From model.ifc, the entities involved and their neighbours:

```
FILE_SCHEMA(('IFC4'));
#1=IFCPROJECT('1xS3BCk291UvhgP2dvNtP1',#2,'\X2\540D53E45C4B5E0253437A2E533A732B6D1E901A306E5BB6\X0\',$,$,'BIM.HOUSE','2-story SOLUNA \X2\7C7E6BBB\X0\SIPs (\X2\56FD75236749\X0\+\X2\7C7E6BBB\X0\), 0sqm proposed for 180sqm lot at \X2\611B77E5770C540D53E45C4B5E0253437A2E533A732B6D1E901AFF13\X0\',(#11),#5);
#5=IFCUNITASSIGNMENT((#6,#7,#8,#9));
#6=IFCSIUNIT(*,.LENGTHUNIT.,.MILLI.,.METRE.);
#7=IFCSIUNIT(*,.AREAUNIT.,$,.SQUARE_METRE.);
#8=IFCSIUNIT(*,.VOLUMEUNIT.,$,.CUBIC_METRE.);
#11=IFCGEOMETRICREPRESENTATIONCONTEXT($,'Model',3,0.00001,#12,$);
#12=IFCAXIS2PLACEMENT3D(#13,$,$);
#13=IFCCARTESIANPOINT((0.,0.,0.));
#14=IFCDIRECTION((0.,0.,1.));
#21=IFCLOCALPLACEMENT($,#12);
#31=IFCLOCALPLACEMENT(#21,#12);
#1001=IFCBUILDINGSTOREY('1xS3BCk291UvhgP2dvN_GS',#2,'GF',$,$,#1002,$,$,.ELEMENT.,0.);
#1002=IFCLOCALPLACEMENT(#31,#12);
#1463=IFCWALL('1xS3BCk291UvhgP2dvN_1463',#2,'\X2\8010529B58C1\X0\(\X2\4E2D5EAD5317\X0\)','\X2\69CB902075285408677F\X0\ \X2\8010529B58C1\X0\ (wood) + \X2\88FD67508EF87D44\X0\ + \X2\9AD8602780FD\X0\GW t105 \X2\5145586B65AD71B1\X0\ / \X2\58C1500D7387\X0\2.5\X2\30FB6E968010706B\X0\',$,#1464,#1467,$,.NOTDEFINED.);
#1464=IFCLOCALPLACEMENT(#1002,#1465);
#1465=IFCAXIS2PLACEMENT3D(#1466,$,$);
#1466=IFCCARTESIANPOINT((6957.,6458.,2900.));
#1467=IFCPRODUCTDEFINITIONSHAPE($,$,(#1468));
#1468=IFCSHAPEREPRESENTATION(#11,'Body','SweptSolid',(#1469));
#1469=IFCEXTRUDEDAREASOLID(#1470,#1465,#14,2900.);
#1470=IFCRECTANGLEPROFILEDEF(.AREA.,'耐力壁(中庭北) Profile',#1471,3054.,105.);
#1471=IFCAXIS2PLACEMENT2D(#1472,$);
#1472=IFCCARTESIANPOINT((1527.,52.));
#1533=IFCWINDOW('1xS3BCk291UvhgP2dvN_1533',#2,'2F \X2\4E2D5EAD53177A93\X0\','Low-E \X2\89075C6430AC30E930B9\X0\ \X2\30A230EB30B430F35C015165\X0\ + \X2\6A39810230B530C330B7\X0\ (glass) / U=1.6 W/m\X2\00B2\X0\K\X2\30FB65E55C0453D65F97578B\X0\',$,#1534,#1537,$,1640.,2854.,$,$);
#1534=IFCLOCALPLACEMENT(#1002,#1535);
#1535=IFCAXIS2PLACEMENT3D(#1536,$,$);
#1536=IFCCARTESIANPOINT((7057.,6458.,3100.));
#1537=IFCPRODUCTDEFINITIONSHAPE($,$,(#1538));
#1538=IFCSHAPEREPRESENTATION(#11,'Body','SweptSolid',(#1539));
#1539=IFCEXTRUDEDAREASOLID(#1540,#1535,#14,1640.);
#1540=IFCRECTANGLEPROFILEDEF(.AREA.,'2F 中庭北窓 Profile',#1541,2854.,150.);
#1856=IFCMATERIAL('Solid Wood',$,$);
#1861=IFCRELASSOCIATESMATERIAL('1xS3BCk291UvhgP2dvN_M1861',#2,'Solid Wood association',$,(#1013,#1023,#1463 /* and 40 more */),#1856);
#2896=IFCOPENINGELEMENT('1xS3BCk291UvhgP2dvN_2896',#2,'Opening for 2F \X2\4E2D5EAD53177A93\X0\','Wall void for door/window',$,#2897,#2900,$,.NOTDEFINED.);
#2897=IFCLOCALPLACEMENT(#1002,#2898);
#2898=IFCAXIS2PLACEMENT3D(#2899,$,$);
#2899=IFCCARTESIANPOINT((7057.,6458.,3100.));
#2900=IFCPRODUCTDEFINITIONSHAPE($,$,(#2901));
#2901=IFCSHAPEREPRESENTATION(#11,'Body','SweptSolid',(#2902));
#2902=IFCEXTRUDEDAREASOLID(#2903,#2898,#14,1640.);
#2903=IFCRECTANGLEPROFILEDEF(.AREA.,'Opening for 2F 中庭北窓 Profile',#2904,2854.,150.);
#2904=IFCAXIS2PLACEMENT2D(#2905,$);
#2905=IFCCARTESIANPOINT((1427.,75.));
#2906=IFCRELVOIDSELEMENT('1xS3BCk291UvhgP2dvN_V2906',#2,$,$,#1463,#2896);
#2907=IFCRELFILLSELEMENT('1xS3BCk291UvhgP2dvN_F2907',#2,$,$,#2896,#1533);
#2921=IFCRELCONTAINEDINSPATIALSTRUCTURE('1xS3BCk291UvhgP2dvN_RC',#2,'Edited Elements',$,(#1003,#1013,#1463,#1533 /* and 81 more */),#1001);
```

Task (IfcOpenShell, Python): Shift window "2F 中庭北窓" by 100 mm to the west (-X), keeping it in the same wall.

```python
import ifcopenshell
import ifcopenshell.api.geometry
import ifcopenshell.util.placement

model = ifcopenshell.open("model.ifc")

window = model.by_guid("1xS3BCk291UvhgP2dvN_1533")
opening = window.FillsVoids[0].RelatingOpeningElement
wall = opening.VoidsElements[0].RelatingBuildingElement

wall_matrix = ifcopenshell.util.placement.get_local_placement(wall.ObjectPlacement)
shift = wall_matrix[:3, 0] * -100.0
before = ifcopenshell.util.placement.get_local_placement(window.ObjectPlacement)[:3, 3].copy()

# The window is not placed relative to its opening, so move both.
for product in (opening, window):
    matrix = ifcopenshell.util.placement.get_local_placement(product.ObjectPlacement)
    matrix[:3, 3] += shift
    ifcopenshell.api.geometry.edit_object_placement(model, product=product, matrix=matrix, is_si=False)

after = ifcopenshell.util.placement.get_local_placement(window.ObjectPlacement)[:3, 3]
print("window moved by", (after - before).round(3) + 0.0)

model.write("model_edited.ifc")
```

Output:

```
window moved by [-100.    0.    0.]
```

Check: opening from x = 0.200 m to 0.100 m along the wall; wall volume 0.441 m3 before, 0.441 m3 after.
